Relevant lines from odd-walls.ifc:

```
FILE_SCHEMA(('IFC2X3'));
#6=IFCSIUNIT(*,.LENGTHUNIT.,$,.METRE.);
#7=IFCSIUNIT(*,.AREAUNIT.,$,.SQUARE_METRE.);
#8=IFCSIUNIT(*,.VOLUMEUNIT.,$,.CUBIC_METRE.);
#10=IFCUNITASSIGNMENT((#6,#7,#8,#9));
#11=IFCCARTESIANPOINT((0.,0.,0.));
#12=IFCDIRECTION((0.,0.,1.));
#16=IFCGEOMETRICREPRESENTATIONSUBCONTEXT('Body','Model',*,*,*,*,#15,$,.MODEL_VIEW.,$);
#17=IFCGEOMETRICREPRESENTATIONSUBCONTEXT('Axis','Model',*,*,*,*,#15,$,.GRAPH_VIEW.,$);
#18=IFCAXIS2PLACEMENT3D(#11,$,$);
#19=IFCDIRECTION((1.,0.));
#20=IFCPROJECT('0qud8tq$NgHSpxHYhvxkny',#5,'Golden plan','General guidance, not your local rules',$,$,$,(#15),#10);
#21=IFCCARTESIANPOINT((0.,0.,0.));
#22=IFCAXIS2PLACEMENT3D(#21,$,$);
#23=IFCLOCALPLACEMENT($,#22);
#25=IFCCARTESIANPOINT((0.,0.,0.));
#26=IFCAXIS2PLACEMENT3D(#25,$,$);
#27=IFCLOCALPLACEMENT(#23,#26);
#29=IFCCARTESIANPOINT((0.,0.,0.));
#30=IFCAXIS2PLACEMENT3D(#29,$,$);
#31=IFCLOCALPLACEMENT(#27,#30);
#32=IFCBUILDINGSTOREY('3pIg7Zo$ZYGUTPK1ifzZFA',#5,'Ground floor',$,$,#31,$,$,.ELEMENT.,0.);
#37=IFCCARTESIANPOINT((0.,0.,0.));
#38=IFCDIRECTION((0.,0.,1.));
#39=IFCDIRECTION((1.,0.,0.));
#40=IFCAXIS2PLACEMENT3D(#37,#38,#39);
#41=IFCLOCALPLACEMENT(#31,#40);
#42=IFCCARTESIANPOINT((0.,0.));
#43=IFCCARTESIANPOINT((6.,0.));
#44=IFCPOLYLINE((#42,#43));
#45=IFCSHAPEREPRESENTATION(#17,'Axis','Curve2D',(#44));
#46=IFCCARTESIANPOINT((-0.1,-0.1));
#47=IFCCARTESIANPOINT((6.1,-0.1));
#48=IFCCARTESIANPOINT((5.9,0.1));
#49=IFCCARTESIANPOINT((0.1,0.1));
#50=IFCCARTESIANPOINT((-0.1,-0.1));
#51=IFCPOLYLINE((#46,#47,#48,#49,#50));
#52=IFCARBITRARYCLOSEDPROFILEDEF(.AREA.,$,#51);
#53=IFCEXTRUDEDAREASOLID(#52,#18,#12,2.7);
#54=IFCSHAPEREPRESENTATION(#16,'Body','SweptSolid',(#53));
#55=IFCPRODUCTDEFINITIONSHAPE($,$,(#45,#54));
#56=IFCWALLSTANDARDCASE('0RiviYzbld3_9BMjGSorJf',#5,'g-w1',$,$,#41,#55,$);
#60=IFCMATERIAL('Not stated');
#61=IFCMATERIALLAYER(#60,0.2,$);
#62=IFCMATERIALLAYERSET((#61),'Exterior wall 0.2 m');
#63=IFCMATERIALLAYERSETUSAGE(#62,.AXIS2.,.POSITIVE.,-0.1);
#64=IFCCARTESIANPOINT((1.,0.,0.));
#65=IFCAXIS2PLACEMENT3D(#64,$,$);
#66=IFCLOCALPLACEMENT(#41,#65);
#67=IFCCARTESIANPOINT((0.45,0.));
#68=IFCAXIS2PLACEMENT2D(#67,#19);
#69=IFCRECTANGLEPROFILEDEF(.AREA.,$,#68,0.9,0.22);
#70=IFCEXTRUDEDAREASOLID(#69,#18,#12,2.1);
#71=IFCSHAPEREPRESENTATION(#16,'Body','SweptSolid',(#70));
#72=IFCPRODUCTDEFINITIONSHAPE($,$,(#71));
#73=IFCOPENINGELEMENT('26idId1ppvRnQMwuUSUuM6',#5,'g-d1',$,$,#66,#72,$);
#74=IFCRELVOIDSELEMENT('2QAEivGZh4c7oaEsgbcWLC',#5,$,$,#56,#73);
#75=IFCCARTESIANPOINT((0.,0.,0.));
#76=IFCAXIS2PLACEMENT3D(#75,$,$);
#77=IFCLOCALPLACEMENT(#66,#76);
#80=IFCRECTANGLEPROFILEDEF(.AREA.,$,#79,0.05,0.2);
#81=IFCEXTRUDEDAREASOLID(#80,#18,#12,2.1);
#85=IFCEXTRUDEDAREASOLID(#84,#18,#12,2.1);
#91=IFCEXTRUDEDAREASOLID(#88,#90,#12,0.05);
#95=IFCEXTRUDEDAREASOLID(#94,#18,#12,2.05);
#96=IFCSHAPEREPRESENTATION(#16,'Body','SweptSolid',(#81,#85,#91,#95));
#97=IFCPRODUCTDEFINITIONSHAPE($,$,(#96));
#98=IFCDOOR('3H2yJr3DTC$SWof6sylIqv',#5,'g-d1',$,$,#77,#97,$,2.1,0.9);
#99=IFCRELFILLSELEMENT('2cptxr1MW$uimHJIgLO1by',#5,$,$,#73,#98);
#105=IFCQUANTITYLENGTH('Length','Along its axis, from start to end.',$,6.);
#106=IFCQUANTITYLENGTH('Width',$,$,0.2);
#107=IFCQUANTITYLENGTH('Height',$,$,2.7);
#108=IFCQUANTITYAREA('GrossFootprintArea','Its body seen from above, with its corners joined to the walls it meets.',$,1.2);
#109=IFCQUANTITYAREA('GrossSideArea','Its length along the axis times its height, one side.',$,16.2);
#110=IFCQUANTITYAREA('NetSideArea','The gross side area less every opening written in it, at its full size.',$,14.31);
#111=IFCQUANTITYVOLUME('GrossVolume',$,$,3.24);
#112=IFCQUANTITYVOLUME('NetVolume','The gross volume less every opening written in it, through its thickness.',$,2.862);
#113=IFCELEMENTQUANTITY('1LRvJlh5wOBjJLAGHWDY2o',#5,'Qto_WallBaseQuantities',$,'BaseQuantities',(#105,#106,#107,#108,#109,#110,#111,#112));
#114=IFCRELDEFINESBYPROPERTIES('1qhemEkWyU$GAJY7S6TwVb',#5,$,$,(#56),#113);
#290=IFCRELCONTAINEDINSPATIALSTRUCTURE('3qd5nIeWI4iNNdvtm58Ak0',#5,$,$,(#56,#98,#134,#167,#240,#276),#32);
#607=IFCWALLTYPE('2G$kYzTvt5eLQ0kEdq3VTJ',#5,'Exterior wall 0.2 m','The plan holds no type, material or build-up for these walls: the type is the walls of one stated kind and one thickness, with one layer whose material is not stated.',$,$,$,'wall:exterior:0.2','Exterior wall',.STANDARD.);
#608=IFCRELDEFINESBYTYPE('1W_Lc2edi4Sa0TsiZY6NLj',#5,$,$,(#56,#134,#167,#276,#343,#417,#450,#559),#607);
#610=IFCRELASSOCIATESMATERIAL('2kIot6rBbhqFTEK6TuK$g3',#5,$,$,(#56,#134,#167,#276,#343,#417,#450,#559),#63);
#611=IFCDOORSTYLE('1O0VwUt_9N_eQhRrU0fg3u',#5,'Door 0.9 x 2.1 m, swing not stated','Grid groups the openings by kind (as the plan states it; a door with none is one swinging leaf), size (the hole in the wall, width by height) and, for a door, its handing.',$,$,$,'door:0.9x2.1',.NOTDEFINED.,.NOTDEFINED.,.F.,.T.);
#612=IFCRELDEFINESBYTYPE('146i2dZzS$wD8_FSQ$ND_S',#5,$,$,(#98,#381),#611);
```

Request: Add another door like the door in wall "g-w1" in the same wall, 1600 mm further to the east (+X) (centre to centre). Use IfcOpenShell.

```python
import ifcopenshell
import ifcopenshell.api.feature
import ifcopenshell.api.geometry
import ifcopenshell.api.pset
import ifcopenshell.api.root
import ifcopenshell.geom
import ifcopenshell.util.element
import ifcopenshell.util.placement
import ifcopenshell.util.shape
import ifcopenshell.util.unit

model = ifcopenshell.open("odd-walls.ifc")
unit_scale = ifcopenshell.util.unit.calculate_unit_scale(model)
area_scale = ifcopenshell.util.unit.calculate_unit_scale(model, "AREAUNIT")
volume_scale = ifcopenshell.util.unit.calculate_unit_scale(model, "VOLUMEUNIT")
settings = ifcopenshell.geom.settings()


def volume(element):
    """Net volume in cubic metres, openings subtracted."""
    shape = ifcopenshell.geom.create_shape(settings, element)
    return ifcopenshell.util.shape.get_volume(shape.geometry)


def reuse_history(source, copy):
    """copy_class also copies each property set's owner history, people and application; keep the originals."""
    for rel in copy.IsDefinedBy:
        if rel.is_a("IfcRelDefinesByProperties") and (history := rel.RelatingPropertyDefinition.OwnerHistory):
            rel.RelatingPropertyDefinition.OwnerHistory = source.OwnerHistory
            ifcopenshell.util.element.remove_deep2(model, history)


door = model.by_guid("3H2yJr3DTC$SWof6sylIqv")
opening = door.FillsVoids[0].RelatingOpeningElement
wall = opening.VoidsElements[0].RelatingBuildingElement
before = volume(wall)
shift = ifcopenshell.util.placement.get_local_placement(wall.ObjectPlacement)[:3, 0] * 1.6 / unit_scale

# copy_class copies the void relationship, type, container and properties, but no geometry.
new_opening = ifcopenshell.api.root.copy_class(model, product=opening)
new_opening.Representation = ifcopenshell.util.element.copy_deep(
    model, opening.Representation, exclude=["IfcGeometricRepresentationContext", "IfcRepresentationMap"]
)
new_door = ifcopenshell.api.root.copy_class(model, product=door)
new_door.Representation = ifcopenshell.util.element.copy_deep(
    model, door.Representation, exclude=["IfcGeometricRepresentationContext", "IfcRepresentationMap"]
)
reuse_history(door, new_door)
fills = ifcopenshell.api.feature.add_filling(model, opening=new_opening, element=new_door)
fills.OwnerHistory = new_door.OwnerHistory  # required in IFC2X3

for old, new in ((opening, new_opening), (door, new_door)):
    matrix = ifcopenshell.util.placement.get_local_placement(old.ObjectPlacement)
    matrix[:3, 3] += shift
    ifcopenshell.api.geometry.edit_object_placement(model, product=new, matrix=matrix, is_si=False)

after = volume(wall)
thickness = 0.2  # wall thickness in metres

# Update the wall's stored quantities.
qto = model.by_id(ifcopenshell.util.element.get_pset(wall, "Qto_WallBaseQuantities", should_inherit=False)["id"])
ifcopenshell.api.pset.edit_qto(model, qto=qto, properties={
    "NetSideArea": after / thickness / area_scale,
    "NetVolume": after / volume_scale,
})

print(f"wall volume {before:.3f} -> {after:.3f} m3")

model.write("odd-walls_edited.ifc")
```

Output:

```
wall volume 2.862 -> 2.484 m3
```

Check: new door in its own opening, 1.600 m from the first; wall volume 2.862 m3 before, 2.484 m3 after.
